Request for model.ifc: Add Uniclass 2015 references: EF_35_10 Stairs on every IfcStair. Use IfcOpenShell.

First a look at what the model holds.

```python
import ifcopenshell

model = ifcopenshell.open("model.ifc")
print(model.schema)
print("classifications:", [c.Name for c in model.by_type("IfcClassification")])
for ifc_class in ("IfcDoor", "IfcRoof", "IfcStair", "IfcWall", "IfcWindow"):
    print(ifc_class, len(model.by_type(ifc_class)))
```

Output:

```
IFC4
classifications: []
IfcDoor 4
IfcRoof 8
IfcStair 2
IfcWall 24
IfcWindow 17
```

```python
import ifcopenshell
import ifcopenshell.api.classification

model = ifcopenshell.open("model.ifc")

system = ifcopenshell.api.classification.add_classification(model, classification="Uniclass 2015")

codes = {
    "IfcStair": ("EF_35_10", "Stairs"),
}
for ifc_class, (code, name) in codes.items():
    products = model.by_type(ifc_class)
    ifcopenshell.api.classification.add_reference(
        model, products=products, classification=system, identification=code, name=name
    )
    print(code, len(products))

model.write("model-out.ifc")
```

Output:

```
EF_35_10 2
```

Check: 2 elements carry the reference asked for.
